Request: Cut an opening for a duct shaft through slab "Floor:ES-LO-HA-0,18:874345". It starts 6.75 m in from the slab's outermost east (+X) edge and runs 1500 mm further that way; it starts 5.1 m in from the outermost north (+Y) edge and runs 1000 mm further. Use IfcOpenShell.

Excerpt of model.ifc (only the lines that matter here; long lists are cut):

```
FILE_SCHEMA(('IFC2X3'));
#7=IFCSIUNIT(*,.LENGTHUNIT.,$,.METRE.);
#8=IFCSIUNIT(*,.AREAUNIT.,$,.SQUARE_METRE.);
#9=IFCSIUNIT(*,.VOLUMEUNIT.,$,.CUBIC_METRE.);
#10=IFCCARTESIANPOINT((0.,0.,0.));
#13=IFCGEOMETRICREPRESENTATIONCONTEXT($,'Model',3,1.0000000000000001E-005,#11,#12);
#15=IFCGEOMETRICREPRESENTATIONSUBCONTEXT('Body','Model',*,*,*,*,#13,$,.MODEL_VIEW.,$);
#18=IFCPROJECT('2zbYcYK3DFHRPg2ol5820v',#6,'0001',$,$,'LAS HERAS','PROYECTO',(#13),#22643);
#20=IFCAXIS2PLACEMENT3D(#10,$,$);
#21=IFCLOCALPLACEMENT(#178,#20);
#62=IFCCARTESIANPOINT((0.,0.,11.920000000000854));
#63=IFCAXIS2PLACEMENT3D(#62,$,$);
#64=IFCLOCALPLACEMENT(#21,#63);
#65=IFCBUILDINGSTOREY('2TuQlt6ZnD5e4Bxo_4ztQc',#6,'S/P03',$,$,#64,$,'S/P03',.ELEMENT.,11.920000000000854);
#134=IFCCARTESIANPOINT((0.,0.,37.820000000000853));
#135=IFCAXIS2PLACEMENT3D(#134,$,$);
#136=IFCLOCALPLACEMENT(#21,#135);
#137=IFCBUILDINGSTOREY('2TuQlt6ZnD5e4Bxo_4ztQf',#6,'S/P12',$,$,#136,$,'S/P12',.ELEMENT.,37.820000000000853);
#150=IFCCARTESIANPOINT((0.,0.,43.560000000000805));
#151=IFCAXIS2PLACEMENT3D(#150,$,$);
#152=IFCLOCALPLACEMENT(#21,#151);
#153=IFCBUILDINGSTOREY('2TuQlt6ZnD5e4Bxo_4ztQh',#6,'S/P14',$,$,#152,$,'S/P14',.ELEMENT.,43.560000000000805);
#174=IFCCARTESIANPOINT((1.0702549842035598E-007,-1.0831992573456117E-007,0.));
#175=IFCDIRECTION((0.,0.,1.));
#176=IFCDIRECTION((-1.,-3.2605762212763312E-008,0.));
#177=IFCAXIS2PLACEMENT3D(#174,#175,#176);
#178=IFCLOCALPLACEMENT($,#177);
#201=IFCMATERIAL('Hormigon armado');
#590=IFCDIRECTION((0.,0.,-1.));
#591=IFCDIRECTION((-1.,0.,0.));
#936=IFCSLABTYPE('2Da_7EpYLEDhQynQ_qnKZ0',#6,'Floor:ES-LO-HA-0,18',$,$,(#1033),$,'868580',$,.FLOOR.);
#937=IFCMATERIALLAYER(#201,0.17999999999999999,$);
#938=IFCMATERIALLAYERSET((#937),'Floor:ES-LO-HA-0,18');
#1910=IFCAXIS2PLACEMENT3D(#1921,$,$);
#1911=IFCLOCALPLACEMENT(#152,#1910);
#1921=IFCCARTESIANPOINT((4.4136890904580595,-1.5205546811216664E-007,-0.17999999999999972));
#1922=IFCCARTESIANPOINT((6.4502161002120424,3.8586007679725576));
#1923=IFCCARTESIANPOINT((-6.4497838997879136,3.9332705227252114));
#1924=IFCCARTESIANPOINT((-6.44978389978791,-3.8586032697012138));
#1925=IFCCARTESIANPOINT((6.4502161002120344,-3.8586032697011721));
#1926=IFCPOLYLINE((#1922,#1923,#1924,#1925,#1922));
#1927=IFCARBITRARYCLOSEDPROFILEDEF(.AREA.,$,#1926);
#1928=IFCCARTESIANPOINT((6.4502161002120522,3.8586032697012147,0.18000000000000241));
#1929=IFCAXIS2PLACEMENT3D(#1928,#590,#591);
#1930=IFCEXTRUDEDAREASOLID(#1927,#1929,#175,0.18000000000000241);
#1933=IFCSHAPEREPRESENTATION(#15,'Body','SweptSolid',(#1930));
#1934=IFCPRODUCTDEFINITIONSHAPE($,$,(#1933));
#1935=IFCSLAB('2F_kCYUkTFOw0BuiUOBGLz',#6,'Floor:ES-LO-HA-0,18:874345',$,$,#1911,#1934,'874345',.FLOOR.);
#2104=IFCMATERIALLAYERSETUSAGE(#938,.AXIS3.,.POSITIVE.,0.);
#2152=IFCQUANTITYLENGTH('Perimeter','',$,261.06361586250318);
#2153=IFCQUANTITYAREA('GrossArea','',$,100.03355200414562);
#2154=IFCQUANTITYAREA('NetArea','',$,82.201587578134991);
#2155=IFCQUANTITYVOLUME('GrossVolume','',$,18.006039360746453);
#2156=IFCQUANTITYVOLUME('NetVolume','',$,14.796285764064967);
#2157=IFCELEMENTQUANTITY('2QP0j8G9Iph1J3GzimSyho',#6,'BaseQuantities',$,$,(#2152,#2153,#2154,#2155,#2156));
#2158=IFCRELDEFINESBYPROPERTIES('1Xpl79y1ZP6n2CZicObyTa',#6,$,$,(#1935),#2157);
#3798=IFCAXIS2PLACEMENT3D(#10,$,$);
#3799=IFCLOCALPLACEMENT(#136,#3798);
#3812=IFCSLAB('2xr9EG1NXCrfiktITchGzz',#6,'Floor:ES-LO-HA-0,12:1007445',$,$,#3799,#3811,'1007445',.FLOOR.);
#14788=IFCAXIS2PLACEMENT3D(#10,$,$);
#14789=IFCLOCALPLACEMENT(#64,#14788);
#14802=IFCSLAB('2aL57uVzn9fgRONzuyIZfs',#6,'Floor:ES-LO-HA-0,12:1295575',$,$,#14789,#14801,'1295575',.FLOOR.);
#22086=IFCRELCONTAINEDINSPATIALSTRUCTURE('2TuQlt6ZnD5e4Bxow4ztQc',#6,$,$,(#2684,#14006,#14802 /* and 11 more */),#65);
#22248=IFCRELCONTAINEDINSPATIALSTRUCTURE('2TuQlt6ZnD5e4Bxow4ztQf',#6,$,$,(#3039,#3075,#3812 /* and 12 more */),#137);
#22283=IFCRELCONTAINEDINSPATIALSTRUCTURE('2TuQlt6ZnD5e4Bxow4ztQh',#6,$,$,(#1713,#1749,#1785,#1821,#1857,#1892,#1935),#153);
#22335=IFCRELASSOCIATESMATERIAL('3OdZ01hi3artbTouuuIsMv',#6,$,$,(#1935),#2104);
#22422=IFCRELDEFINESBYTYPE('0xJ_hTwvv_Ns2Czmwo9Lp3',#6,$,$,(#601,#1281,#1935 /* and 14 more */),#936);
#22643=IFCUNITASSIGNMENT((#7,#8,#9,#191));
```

```python
import numpy as np
import ifcopenshell
import ifcopenshell.api.feature
import ifcopenshell.api.geometry
import ifcopenshell.api.pset
import ifcopenshell.api.root
import ifcopenshell.geom
import ifcopenshell.util.element
import ifcopenshell.util.placement
import ifcopenshell.util.representation
import ifcopenshell.util.shape
import ifcopenshell.util.unit

model = ifcopenshell.open("model.ifc")
unit_scale = ifcopenshell.util.unit.calculate_unit_scale(model)
area_scale = ifcopenshell.util.unit.calculate_unit_scale(model, "AREAUNIT")
volume_scale = ifcopenshell.util.unit.calculate_unit_scale(model, "VOLUMEUNIT")
settings = ifcopenshell.geom.settings()


def volume(element):
    """Net volume in cubic metres, openings subtracted."""
    shape = ifcopenshell.geom.create_shape(settings, element)
    return ifcopenshell.util.shape.get_volume(shape.geometry)


slab = model.by_id(1935)
before = volume(slab)

# Extent in the slab's own axes, in metres. The edges named are its -X and -Y sides.
slab_shape = ifcopenshell.geom.create_shape(settings, slab)
vertices = ifcopenshell.util.shape.get_vertices(slab_shape.geometry)
x_min, y_min, bottom = vertices.min(axis=0)
top = vertices[:, 2].max()

opening = ifcopenshell.api.root.create_entity(model, ifc_class="IfcOpeningElement", name="Duct shaft opening")
context = ifcopenshell.util.representation.get_context(model, "Model", "Body", "MODEL_VIEW")
width, depth = 1.5, 1
outline = [(0.0, 0.0), (width, 0.0), (width, depth), (0.0, depth), (0.0, 0.0)]
# Overshoot both faces by 50 mm so the cut is clean.
shape = ifcopenshell.api.geometry.add_slab_representation(
    model, context=context, depth=top - bottom + 0.1, polyline=outline
)
ifcopenshell.api.geometry.assign_representation(model, product=opening, representation=shape)

matrix = ifcopenshell.util.placement.get_local_placement(slab.ObjectPlacement)
matrix[:, 3] = matrix @ np.append(np.array([x_min + 6.75, y_min + 5.1, bottom - 0.05]) / unit_scale, 1.0)
ifcopenshell.api.geometry.edit_object_placement(model, product=opening, matrix=matrix, is_si=False)
ifcopenshell.api.feature.add_feature(model, feature=opening, element=slab)

after = volume(slab)

# Update the slab's stored quantities.
qto = model.by_id(ifcopenshell.util.element.get_pset(slab, "BaseQuantities", should_inherit=False)["id"])
ifcopenshell.api.pset.edit_qto(model, qto=qto, properties={
    "NetArea": after / (top - bottom) / area_scale,
    "NetVolume": after / volume_scale,
})

print(f"slab volume {before:.3f} -> {after:.3f} m3")

model.write("model_v2.ifc")
```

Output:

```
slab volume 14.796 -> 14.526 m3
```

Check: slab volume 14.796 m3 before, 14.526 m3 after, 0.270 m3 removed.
